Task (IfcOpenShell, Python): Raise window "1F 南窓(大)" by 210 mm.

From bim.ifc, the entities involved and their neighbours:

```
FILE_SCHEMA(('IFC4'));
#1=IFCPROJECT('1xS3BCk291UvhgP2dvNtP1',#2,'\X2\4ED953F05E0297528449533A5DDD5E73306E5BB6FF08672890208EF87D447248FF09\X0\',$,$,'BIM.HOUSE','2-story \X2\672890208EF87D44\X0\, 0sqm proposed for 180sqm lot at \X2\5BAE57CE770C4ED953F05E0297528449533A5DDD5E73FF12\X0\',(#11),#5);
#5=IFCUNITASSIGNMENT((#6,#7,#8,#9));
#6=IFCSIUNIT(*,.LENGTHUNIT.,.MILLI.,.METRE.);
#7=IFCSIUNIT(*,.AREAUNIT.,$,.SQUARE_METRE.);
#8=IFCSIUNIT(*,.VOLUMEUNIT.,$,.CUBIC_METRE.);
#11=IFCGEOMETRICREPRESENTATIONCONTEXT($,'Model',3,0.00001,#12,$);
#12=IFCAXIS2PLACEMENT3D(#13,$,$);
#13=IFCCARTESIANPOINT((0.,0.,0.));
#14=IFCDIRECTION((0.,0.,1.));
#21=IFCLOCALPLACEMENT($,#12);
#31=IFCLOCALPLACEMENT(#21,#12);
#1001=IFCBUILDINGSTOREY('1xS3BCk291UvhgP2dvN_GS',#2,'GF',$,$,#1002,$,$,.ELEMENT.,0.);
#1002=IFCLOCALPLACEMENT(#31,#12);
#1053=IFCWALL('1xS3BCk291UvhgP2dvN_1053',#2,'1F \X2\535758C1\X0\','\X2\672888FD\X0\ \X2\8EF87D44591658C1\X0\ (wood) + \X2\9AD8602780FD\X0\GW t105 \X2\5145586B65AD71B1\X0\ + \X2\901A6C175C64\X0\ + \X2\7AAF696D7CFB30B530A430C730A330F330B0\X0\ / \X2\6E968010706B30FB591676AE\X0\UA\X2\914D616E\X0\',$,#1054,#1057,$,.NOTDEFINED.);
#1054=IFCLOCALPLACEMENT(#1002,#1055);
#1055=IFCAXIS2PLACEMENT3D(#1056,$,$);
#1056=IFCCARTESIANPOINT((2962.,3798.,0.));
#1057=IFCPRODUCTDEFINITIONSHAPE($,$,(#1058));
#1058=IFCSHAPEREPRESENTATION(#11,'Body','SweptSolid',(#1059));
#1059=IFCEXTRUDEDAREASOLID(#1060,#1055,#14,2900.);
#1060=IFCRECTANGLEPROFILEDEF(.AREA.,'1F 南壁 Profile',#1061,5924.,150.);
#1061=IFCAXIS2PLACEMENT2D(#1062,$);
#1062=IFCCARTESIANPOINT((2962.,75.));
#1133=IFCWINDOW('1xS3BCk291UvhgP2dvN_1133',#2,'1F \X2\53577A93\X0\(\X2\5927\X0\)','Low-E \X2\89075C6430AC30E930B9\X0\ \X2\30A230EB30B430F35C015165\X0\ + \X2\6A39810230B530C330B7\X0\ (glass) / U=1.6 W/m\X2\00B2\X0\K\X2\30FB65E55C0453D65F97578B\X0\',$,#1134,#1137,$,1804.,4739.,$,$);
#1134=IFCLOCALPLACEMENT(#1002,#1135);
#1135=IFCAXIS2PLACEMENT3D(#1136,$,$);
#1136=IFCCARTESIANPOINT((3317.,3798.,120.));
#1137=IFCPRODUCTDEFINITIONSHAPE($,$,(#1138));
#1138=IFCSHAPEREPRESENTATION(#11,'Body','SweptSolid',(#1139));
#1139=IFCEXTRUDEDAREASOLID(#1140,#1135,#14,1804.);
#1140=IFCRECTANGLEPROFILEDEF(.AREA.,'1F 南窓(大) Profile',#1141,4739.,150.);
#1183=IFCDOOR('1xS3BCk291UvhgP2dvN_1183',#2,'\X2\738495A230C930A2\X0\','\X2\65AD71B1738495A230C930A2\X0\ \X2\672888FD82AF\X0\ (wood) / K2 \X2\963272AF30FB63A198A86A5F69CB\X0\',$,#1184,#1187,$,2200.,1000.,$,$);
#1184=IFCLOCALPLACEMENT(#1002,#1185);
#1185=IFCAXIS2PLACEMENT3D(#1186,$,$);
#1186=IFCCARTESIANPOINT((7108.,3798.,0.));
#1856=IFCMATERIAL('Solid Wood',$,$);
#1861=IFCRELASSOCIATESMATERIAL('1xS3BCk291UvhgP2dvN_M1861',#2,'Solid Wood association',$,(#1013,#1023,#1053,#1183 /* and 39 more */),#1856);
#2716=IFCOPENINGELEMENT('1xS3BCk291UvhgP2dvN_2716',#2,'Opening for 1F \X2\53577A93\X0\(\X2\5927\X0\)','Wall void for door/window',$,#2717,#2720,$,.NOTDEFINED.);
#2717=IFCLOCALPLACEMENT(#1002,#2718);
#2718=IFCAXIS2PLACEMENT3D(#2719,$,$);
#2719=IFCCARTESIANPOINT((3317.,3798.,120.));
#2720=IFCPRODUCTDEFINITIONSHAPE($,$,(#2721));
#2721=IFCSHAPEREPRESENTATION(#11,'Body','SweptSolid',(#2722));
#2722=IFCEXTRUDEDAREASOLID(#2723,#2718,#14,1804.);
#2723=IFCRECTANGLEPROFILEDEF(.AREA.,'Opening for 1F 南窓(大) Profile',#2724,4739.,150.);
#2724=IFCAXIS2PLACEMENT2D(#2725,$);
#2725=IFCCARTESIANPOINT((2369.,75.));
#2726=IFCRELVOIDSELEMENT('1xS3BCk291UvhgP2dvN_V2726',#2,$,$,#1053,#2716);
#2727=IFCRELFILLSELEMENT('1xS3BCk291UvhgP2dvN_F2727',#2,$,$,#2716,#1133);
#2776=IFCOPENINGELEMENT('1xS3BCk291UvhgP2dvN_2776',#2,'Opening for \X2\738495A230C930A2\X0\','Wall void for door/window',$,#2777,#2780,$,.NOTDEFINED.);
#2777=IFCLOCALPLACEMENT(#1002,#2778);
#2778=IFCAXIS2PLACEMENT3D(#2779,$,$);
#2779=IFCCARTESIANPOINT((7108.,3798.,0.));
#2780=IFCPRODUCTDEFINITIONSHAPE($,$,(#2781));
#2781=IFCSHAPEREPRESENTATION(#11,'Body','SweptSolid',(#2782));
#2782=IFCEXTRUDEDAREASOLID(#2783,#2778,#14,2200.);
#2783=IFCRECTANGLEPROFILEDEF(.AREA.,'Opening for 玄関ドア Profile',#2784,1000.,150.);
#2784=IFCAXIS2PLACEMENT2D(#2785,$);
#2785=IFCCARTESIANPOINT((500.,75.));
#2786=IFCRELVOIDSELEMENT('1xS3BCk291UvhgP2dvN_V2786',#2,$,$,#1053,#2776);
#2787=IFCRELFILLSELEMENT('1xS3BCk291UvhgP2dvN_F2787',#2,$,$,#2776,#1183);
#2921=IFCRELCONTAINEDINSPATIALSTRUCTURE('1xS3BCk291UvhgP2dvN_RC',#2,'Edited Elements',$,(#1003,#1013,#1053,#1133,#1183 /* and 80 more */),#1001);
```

```python
import numpy as np
import ifcopenshell
import ifcopenshell.api.geometry
import ifcopenshell.util.placement
import ifcopenshell.util.unit

model = ifcopenshell.open("bim.ifc")
unit_scale = ifcopenshell.util.unit.calculate_unit_scale(model)

window = model.by_guid("1xS3BCk291UvhgP2dvN_1133")
opening = window.FillsVoids[0].RelatingOpeningElement
dz = 0.21 / unit_scale

shift = np.array([0.0, 0.0, dz])
# The window is not placed relative to its opening, so move both.
for product in (opening, window):
    matrix = ifcopenshell.util.placement.get_local_placement(product.ObjectPlacement)
    matrix[:3, 3] += shift
    ifcopenshell.api.geometry.edit_object_placement(model, product=product, matrix=matrix, is_si=False)

print(f"moved by {dz * unit_scale:+.3f} m")

model.write("bim-out.ifc")
```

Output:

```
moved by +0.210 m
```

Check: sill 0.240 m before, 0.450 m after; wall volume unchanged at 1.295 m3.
